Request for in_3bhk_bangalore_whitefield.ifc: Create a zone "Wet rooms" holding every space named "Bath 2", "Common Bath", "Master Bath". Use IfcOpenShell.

First a look at what the model holds.

```python
import ifcopenshell

model = ifcopenshell.open("in_3bhk_bangalore_whitefield.ifc")
print(model.schema)
seen = {}
for space in model.by_type("IfcSpace"):
    seen[space.LongName] = seen.get(space.LongName, 0) + 1
for name, count in sorted(seen.items(), key=str):
    print(count, "x", name)
print("zones:", [z.Name for z in model.by_type("IfcZone")][:20])
```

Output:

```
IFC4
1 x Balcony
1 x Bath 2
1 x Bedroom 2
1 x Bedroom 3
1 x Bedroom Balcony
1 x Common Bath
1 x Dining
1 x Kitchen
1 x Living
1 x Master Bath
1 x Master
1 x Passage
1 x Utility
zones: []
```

```python
import ifcopenshell
import ifcopenshell.api.group
import ifcopenshell.api.root

model = ifcopenshell.open("in_3bhk_bangalore_whitefield.ifc")

names = {"Bath 2", "Common Bath", "Master Bath"}
spaces = [s for s in model.by_type("IfcSpace") if s.LongName in names]

zone = ifcopenshell.api.root.create_entity(model, ifc_class="IfcZone", name="Wet rooms")
ifcopenshell.api.group.assign_group(model, products=spaces, group=zone)
print(len(spaces), "spaces in", zone.Name)

model.write("in_3bhk_bangalore_whitefield_edited.ifc")
```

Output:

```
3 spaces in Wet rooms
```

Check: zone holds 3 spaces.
